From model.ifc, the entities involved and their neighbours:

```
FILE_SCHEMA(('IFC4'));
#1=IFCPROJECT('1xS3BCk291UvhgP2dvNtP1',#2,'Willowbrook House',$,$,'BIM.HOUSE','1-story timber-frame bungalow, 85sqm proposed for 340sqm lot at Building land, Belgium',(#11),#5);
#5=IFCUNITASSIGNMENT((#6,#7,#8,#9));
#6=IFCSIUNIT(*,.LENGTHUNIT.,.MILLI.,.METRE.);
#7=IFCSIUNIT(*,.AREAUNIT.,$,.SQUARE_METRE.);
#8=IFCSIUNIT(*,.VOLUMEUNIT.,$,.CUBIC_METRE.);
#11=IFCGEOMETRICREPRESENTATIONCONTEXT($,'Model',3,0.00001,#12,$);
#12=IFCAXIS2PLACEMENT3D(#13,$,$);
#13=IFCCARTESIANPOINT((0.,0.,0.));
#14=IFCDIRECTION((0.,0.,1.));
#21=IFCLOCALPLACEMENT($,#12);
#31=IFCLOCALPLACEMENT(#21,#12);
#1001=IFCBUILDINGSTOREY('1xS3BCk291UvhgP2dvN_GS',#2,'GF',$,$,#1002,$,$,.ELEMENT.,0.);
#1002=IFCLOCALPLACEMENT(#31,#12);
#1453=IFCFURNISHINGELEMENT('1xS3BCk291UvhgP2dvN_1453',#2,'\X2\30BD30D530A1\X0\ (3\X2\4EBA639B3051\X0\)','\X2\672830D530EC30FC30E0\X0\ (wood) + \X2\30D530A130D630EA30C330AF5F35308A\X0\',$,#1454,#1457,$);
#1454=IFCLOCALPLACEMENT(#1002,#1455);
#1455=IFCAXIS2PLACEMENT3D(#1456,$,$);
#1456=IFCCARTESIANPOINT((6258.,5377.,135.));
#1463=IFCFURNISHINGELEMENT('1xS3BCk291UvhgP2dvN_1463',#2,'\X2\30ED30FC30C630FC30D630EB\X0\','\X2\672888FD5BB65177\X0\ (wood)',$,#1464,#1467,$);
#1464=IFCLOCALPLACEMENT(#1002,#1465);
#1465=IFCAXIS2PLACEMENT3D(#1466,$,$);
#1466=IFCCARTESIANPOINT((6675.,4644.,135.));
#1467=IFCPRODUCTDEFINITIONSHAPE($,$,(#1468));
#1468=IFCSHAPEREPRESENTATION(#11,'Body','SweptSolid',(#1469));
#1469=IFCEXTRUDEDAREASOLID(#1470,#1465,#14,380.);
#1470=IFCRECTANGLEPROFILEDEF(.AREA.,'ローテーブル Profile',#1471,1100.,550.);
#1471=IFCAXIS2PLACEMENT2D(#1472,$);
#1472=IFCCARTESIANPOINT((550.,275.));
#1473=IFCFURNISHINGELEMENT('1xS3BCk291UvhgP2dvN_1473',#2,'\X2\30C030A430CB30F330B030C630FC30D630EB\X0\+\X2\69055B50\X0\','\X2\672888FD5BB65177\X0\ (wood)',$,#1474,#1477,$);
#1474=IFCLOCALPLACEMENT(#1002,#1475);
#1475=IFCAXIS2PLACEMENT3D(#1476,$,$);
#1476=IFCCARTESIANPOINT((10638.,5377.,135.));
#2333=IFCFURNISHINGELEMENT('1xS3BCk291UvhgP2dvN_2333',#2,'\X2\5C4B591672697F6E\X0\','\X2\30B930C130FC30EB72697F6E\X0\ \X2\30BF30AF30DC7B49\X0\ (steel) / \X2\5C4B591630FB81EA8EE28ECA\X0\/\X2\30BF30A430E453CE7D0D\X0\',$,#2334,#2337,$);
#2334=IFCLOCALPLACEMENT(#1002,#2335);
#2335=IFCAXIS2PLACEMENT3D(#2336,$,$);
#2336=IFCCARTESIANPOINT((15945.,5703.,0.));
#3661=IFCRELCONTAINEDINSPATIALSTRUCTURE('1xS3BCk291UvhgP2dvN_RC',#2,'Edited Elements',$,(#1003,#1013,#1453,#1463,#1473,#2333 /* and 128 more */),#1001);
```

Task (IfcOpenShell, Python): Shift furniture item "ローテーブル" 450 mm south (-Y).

```python
import ifcopenshell
import ifcopenshell.api.geometry
import ifcopenshell.util.placement

model = ifcopenshell.open("model.ifc")

item = model.by_id(1463)
matrix = ifcopenshell.util.placement.get_local_placement(item.ObjectPlacement)
matrix[1, 3] -= 450.0
ifcopenshell.api.geometry.edit_object_placement(model, product=item, matrix=matrix, is_si=False)

print(ifcopenshell.util.placement.get_local_placement(item.ObjectPlacement).round(3) + 0.0)

model.write("model_rev.ifc")
```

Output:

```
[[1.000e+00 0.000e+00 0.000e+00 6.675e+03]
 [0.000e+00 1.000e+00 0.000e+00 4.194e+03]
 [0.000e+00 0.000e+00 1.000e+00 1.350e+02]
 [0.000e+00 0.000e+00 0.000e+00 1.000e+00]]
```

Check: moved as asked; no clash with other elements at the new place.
